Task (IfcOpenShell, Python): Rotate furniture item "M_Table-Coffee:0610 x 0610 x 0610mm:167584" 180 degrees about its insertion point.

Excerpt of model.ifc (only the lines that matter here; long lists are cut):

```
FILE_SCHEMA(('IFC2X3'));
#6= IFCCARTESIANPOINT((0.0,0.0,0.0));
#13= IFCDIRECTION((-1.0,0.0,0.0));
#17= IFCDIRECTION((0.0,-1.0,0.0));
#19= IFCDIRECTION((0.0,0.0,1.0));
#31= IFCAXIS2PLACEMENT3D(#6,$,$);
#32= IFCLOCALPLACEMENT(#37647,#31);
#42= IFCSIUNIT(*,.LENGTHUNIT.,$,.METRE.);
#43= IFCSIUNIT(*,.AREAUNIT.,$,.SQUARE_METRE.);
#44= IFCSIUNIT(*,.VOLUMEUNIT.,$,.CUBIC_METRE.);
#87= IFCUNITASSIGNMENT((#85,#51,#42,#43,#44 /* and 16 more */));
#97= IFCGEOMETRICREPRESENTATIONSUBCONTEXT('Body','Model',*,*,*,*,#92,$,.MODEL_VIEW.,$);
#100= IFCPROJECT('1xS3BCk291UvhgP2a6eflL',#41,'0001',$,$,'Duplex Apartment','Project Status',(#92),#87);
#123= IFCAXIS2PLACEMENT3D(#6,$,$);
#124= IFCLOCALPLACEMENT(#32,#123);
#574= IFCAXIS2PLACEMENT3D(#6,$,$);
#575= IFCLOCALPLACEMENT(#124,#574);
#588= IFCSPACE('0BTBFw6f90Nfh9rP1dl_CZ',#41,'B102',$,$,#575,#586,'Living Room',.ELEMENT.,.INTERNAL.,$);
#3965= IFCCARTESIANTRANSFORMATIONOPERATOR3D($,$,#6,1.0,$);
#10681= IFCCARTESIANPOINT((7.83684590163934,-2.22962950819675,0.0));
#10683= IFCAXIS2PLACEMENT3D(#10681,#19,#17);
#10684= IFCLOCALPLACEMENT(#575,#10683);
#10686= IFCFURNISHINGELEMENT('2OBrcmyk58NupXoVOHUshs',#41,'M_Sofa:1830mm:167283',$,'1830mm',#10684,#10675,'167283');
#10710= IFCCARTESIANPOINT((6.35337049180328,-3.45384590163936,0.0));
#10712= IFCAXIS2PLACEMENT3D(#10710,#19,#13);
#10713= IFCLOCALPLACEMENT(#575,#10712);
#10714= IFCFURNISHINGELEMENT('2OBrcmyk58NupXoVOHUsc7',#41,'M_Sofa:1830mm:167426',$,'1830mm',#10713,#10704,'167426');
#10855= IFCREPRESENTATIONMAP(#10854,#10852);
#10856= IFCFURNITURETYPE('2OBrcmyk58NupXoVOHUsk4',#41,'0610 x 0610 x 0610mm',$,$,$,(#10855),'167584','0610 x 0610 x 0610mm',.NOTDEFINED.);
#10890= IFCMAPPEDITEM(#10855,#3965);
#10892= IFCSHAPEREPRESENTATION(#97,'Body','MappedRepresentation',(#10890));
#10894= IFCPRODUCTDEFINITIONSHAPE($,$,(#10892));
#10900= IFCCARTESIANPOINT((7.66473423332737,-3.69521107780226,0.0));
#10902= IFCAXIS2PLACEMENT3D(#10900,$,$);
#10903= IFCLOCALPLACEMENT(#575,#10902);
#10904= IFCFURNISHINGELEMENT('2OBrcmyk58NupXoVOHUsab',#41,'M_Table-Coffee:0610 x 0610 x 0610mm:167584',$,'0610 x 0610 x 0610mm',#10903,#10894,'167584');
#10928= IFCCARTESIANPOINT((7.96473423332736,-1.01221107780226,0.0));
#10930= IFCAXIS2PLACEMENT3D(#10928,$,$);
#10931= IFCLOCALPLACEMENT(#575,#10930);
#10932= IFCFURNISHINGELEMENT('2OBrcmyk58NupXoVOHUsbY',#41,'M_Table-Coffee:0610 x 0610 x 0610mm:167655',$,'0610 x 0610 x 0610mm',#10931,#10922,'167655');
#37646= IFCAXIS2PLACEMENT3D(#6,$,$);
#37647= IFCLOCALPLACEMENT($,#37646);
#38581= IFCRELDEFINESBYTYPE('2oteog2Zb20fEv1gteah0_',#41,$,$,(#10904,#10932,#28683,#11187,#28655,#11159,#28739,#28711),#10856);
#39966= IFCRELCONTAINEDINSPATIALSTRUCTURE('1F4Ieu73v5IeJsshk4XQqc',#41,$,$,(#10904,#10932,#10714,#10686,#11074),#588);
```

```python
import ifcopenshell
import ifcopenshell.api.geometry
import ifcopenshell.util.placement

model = ifcopenshell.open("model.ifc")

item = model.by_guid("2OBrcmyk58NupXoVOHUsab")
matrix = ifcopenshell.util.placement.get_local_placement(item.ObjectPlacement)
matrix = matrix @ ifcopenshell.util.placement.rotation(180, "Z")
ifcopenshell.api.geometry.edit_object_placement(model, product=item, matrix=matrix, is_si=False)

print(ifcopenshell.util.placement.get_local_placement(item.ObjectPlacement).round(3) + 0.0)

model.write("model_v2.ifc")
```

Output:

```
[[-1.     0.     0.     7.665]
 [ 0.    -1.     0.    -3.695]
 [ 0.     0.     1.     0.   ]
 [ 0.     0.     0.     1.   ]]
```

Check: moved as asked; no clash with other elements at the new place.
